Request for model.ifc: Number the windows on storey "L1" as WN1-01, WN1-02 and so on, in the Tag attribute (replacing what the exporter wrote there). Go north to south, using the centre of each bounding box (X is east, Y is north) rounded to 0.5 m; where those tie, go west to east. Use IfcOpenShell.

First a look at what the model holds.

```python
import ifcopenshell
import ifcopenshell.util.element
import ifcopenshell.util.placement

model = ifcopenshell.open("model.ifc")
print(model.schema)
storey = next(s for s in model.by_type("IfcBuildingStorey") if s.Name == "L1")
windows = [e for e in ifcopenshell.util.element.get_decomposition(storey) if e.is_a("IfcWindow")]
for e in sorted(windows, key=lambda e: e.id()):
    origin = ifcopenshell.util.placement.get_local_placement(e.ObjectPlacement)[:3, 3]
    print(e.id(), e.Tag, e.Name, origin.round(2) + 0.0, sep=" | ")
```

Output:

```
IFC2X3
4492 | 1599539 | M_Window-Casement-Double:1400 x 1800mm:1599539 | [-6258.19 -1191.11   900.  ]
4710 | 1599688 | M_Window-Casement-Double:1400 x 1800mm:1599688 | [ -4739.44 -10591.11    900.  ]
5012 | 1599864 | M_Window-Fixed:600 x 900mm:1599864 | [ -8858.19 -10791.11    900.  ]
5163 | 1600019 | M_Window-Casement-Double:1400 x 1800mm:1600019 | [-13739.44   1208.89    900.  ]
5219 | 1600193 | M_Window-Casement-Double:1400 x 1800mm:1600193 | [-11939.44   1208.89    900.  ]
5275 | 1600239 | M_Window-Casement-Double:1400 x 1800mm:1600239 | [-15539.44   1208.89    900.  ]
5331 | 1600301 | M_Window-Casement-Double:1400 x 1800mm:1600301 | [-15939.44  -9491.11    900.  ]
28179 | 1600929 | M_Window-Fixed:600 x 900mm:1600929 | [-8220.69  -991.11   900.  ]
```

```python
import ifcopenshell
import ifcopenshell.geom
import ifcopenshell.util.element
import ifcopenshell.util.shape

model = ifcopenshell.open("model.ifc")
settings = ifcopenshell.geom.settings()
settings.set("use-world-coords", True)


def centre(element):
    shape = ifcopenshell.geom.create_shape(settings, element)
    return ifcopenshell.util.shape.get_bbox_centroid(shape.geometry)


storey = next(s for s in model.by_type("IfcBuildingStorey") if s.Name == "L1")
windows = [e for e in ifcopenshell.util.element.get_decomposition(storey) if e.is_a("IfcWindow")]

# Insertion points can sit at a corner or the storey origin, so sort by the geometry (in metres).
centres = {e: centre(e) for e in windows}
windows.sort(key=lambda e: (-round(centres[e][1] / 0.5), centres[e][0]))

for i, e in enumerate(windows, start=1):
    number = f"WN1-{i:02d}"
    e.Tag = number
    print(e.id(), number)

model.write("model_v2.ifc")
```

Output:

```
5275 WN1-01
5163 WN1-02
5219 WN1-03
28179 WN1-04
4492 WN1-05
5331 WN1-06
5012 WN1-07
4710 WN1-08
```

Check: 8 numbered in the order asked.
